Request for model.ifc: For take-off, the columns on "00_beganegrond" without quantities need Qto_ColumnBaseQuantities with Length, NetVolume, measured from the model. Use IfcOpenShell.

First a look at what the model holds.

```python
import ifcopenshell
import ifcopenshell.util.element
import ifcopenshell.util.unit

model = ifcopenshell.open("model.ifc")
print(model.schema)
for unit_type in ("LENGTHUNIT", "AREAUNIT", "VOLUMEUNIT"):
    print(unit_type, ifcopenshell.util.unit.calculate_unit_scale(model, unit_type))
storey = next(s for s in model.by_type("IfcBuildingStorey") if s.Name == "00_beganegrond")
columns = [e for e in ifcopenshell.util.element.get_decomposition(storey) if e.is_a("IfcColumn")]
for e in sorted(columns, key=lambda e: e.id()):
    print(e.id(), e.is_a(), e.Name, list(ifcopenshell.util.element.get_psets(e, qtos_only=True)), sep=" | ")
```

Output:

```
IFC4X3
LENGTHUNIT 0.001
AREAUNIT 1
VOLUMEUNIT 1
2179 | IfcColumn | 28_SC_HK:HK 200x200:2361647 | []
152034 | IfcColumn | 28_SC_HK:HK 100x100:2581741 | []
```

```python
import ifcopenshell
import ifcopenshell.api.pset
import ifcopenshell.geom
import ifcopenshell.util.element
import ifcopenshell.util.shape
import ifcopenshell.util.unit

model = ifcopenshell.open("model.ifc")
unit_scale = ifcopenshell.util.unit.calculate_unit_scale(model)
volume_scale = ifcopenshell.util.unit.calculate_unit_scale(model, "VOLUMEUNIT")
settings = ifcopenshell.geom.settings()

storey = next(s for s in model.by_type("IfcBuildingStorey") if s.Name == "00_beganegrond")
columns = [e for e in ifcopenshell.util.element.get_decomposition(storey) if e.is_a("IfcColumn")]

for e in sorted(columns, key=lambda e: e.id()):
    if ifcopenshell.util.element.get_psets(e, qtos_only=True, should_inherit=False):
        continue
    # Geometry comes back in metres, in the element's own axes.
    shape = ifcopenshell.geom.create_shape(settings, e)
    values = {
        "Length": ifcopenshell.util.shape.get_z(shape.geometry) / unit_scale,
        "NetVolume": ifcopenshell.util.shape.get_volume(shape.geometry) / volume_scale,
    }
    qto = ifcopenshell.api.pset.add_qto(model, product=e, name="Qto_ColumnBaseQuantities")
    ifcopenshell.api.pset.edit_qto(model, qto=qto, properties=values)
    print(e.id(), {k: round(v, 3) for k, v in values.items()})

model.write("model_v2.ifc")
```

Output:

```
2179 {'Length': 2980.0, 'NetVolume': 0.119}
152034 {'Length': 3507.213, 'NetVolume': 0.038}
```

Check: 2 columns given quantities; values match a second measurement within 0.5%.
